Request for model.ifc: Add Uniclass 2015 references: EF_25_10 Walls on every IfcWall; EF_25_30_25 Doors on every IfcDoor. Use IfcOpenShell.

First a look at what the model holds.

```python
import ifcopenshell

model = ifcopenshell.open("model.ifc")
print(model.schema)
print("classifications:", [c.Name for c in model.by_type("IfcClassification")])
for ifc_class in ("IfcDoor", "IfcRoof", "IfcStair", "IfcWall", "IfcWindow"):
    print(ifc_class, len(model.by_type(ifc_class)))
```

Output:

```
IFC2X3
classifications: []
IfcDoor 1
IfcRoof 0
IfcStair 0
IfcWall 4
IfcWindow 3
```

```python
import ifcopenshell
import ifcopenshell.api.classification

model = ifcopenshell.open("model.ifc")

# IFC2X3 requires Source and Edition and has no link from the project to the system.
system = model.create_entity("IfcClassification", Source="NBS", Edition="2015", Name="Uniclass 2015")

codes = {
    "IfcWall": ("EF_25_10", "Walls"),
    "IfcDoor": ("EF_25_30_25", "Doors"),
}
for ifc_class, (code, name) in codes.items():
    products = model.by_type(ifc_class)
    ifcopenshell.api.classification.add_reference(
        model, products=products, classification=system, identification=code, name=name
    )
    print(code, len(products))

model.write("model_v2.ifc")
```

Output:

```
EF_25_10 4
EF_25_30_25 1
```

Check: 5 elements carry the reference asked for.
